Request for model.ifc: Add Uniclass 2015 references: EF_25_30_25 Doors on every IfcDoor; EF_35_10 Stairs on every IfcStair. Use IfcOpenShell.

First a look at what the model holds.

```python
import ifcopenshell

model = ifcopenshell.open("model.ifc")
print(model.schema)
print("classifications:", [c.Name for c in model.by_type("IfcClassification")])
for ifc_class in ("IfcDoor", "IfcRoof", "IfcStair", "IfcWall", "IfcWindow"):
    print(ifc_class, len(model.by_type(ifc_class)))
```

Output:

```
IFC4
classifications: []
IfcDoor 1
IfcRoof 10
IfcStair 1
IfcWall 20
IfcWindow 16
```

```python
import ifcopenshell
import ifcopenshell.api.classification

model = ifcopenshell.open("model.ifc")

system = ifcopenshell.api.classification.add_classification(model, classification="Uniclass 2015")

codes = {
    "IfcDoor": ("EF_25_30_25", "Doors"),
    "IfcStair": ("EF_35_10", "Stairs"),
}
for ifc_class, (code, name) in codes.items():
    products = model.by_type(ifc_class)
    ifcopenshell.api.classification.add_reference(
        model, products=products, classification=system, identification=code, name=name
    )
    print(code, len(products))

model.write("model_v2.ifc")
```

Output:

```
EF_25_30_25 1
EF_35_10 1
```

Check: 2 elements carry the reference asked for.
